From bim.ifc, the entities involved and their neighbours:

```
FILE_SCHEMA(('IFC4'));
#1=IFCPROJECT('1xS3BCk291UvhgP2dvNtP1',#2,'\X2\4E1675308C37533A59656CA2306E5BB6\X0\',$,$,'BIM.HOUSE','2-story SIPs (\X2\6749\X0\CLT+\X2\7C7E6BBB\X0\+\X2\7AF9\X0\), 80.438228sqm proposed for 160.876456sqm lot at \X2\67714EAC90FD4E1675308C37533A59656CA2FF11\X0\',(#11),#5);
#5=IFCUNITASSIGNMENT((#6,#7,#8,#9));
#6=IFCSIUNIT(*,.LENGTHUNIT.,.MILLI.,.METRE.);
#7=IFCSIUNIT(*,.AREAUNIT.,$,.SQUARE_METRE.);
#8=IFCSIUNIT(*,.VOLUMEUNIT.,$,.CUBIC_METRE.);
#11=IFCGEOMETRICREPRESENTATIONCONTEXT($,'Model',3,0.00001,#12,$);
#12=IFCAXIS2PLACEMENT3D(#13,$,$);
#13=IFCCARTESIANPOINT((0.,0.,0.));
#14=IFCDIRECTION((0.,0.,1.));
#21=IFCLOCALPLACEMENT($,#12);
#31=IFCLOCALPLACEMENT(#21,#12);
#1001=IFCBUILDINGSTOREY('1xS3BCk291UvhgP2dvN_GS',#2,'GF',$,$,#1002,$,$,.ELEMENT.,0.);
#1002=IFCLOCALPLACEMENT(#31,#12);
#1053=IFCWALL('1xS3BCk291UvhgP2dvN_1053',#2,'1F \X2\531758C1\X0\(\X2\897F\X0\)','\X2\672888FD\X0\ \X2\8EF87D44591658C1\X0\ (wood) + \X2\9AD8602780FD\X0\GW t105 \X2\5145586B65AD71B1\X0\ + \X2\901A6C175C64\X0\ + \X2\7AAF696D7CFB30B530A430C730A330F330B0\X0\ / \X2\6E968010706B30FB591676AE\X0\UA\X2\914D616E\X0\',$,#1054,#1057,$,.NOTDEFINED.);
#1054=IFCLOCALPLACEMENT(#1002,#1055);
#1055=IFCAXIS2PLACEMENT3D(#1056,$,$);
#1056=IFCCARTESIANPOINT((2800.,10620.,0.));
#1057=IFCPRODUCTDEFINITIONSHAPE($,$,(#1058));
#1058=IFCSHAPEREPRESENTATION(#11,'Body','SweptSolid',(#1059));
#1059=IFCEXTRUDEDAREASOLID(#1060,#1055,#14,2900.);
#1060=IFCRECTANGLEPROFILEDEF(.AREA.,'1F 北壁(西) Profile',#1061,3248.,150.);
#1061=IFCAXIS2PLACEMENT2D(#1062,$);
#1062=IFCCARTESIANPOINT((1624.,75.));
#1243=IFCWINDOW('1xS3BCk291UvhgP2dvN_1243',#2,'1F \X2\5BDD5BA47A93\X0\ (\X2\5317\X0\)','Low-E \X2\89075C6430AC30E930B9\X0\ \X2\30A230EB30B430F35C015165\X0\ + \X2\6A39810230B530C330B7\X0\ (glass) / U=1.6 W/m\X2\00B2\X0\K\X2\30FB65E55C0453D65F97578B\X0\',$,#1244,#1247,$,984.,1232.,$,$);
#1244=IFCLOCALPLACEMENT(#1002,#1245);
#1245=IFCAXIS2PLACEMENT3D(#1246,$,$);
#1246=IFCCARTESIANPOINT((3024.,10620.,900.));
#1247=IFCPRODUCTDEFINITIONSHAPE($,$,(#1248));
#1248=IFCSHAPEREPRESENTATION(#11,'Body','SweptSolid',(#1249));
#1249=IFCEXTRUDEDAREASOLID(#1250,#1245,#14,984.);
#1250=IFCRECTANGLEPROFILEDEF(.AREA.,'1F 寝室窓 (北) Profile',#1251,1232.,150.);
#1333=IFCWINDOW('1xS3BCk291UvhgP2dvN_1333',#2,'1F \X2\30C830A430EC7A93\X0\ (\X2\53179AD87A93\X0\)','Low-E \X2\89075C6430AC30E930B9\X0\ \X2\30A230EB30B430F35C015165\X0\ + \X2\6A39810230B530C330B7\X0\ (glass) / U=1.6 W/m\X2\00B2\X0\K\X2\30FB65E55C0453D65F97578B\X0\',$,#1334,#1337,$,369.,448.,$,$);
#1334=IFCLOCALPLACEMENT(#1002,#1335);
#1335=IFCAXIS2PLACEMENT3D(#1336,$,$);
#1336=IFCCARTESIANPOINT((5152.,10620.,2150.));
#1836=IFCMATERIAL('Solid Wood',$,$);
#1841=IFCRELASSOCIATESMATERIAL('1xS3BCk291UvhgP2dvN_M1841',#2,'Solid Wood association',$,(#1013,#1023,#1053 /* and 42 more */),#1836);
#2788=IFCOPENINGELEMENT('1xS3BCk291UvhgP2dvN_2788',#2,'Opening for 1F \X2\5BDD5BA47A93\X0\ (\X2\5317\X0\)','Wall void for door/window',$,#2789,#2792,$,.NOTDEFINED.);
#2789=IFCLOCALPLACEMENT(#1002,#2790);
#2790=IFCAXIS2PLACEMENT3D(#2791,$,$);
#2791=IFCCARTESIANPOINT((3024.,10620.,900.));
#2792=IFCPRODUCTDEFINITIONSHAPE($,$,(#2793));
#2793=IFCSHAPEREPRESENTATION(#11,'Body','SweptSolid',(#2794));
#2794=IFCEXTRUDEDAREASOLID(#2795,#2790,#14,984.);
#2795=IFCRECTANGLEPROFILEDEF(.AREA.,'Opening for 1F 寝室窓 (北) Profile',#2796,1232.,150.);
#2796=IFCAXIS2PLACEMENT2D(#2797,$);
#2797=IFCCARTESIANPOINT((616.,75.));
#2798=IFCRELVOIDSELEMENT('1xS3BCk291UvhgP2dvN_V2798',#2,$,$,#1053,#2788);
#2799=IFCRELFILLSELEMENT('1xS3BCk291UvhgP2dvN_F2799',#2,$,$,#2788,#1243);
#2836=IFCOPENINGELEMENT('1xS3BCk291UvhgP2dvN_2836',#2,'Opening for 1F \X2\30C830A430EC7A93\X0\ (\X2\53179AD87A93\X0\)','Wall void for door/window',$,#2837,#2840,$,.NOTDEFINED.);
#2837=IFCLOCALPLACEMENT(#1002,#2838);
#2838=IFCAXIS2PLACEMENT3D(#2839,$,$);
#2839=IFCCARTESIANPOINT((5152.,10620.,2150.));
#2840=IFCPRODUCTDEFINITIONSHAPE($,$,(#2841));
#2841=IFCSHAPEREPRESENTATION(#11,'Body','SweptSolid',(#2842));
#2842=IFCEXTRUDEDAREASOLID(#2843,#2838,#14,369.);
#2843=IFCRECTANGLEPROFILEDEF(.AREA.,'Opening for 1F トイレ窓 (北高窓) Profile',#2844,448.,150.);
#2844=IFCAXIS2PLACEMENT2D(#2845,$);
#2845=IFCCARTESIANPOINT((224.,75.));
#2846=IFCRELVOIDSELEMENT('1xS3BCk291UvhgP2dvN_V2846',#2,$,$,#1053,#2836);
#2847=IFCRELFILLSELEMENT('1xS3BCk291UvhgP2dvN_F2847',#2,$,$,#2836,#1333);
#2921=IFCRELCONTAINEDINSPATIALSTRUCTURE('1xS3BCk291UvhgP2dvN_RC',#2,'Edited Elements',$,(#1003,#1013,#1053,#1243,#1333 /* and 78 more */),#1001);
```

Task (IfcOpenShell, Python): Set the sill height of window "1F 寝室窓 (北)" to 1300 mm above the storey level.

```python
import numpy as np
import ifcopenshell
import ifcopenshell.api.geometry
import ifcopenshell.geom
import ifcopenshell.util.element
import ifcopenshell.util.placement
import ifcopenshell.util.shape
import ifcopenshell.util.unit

model = ifcopenshell.open("bim.ifc")
unit_scale = ifcopenshell.util.unit.calculate_unit_scale(model)

window = model.by_id(1243)
opening = window.FillsVoids[0].RelatingOpeningElement
storey = ifcopenshell.util.element.get_container(window, ifc_class="IfcBuildingStorey")
level = ifcopenshell.util.placement.get_local_placement(storey.ObjectPlacement)[2, 3]

# The opening's origin need not be at the sill, so measure its lowest point.
shape = ifcopenshell.geom.create_shape(ifcopenshell.geom.settings(), opening)
bottom = ifcopenshell.util.shape.get_shape_bottom_elevation(shape, shape.geometry) / unit_scale
dz = level + 1.3 / unit_scale - bottom

shift = np.array([0.0, 0.0, dz])
# The window is not placed relative to its opening, so move both.
for product in (opening, window):
    matrix = ifcopenshell.util.placement.get_local_placement(product.ObjectPlacement)
    matrix[:3, 3] += shift
    ifcopenshell.api.geometry.edit_object_placement(model, product=product, matrix=matrix, is_si=False)

print(f"moved by {dz * unit_scale:+.3f} m")

model.write("bim_rev.ifc")
```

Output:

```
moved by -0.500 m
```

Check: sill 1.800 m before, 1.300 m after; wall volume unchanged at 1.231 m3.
